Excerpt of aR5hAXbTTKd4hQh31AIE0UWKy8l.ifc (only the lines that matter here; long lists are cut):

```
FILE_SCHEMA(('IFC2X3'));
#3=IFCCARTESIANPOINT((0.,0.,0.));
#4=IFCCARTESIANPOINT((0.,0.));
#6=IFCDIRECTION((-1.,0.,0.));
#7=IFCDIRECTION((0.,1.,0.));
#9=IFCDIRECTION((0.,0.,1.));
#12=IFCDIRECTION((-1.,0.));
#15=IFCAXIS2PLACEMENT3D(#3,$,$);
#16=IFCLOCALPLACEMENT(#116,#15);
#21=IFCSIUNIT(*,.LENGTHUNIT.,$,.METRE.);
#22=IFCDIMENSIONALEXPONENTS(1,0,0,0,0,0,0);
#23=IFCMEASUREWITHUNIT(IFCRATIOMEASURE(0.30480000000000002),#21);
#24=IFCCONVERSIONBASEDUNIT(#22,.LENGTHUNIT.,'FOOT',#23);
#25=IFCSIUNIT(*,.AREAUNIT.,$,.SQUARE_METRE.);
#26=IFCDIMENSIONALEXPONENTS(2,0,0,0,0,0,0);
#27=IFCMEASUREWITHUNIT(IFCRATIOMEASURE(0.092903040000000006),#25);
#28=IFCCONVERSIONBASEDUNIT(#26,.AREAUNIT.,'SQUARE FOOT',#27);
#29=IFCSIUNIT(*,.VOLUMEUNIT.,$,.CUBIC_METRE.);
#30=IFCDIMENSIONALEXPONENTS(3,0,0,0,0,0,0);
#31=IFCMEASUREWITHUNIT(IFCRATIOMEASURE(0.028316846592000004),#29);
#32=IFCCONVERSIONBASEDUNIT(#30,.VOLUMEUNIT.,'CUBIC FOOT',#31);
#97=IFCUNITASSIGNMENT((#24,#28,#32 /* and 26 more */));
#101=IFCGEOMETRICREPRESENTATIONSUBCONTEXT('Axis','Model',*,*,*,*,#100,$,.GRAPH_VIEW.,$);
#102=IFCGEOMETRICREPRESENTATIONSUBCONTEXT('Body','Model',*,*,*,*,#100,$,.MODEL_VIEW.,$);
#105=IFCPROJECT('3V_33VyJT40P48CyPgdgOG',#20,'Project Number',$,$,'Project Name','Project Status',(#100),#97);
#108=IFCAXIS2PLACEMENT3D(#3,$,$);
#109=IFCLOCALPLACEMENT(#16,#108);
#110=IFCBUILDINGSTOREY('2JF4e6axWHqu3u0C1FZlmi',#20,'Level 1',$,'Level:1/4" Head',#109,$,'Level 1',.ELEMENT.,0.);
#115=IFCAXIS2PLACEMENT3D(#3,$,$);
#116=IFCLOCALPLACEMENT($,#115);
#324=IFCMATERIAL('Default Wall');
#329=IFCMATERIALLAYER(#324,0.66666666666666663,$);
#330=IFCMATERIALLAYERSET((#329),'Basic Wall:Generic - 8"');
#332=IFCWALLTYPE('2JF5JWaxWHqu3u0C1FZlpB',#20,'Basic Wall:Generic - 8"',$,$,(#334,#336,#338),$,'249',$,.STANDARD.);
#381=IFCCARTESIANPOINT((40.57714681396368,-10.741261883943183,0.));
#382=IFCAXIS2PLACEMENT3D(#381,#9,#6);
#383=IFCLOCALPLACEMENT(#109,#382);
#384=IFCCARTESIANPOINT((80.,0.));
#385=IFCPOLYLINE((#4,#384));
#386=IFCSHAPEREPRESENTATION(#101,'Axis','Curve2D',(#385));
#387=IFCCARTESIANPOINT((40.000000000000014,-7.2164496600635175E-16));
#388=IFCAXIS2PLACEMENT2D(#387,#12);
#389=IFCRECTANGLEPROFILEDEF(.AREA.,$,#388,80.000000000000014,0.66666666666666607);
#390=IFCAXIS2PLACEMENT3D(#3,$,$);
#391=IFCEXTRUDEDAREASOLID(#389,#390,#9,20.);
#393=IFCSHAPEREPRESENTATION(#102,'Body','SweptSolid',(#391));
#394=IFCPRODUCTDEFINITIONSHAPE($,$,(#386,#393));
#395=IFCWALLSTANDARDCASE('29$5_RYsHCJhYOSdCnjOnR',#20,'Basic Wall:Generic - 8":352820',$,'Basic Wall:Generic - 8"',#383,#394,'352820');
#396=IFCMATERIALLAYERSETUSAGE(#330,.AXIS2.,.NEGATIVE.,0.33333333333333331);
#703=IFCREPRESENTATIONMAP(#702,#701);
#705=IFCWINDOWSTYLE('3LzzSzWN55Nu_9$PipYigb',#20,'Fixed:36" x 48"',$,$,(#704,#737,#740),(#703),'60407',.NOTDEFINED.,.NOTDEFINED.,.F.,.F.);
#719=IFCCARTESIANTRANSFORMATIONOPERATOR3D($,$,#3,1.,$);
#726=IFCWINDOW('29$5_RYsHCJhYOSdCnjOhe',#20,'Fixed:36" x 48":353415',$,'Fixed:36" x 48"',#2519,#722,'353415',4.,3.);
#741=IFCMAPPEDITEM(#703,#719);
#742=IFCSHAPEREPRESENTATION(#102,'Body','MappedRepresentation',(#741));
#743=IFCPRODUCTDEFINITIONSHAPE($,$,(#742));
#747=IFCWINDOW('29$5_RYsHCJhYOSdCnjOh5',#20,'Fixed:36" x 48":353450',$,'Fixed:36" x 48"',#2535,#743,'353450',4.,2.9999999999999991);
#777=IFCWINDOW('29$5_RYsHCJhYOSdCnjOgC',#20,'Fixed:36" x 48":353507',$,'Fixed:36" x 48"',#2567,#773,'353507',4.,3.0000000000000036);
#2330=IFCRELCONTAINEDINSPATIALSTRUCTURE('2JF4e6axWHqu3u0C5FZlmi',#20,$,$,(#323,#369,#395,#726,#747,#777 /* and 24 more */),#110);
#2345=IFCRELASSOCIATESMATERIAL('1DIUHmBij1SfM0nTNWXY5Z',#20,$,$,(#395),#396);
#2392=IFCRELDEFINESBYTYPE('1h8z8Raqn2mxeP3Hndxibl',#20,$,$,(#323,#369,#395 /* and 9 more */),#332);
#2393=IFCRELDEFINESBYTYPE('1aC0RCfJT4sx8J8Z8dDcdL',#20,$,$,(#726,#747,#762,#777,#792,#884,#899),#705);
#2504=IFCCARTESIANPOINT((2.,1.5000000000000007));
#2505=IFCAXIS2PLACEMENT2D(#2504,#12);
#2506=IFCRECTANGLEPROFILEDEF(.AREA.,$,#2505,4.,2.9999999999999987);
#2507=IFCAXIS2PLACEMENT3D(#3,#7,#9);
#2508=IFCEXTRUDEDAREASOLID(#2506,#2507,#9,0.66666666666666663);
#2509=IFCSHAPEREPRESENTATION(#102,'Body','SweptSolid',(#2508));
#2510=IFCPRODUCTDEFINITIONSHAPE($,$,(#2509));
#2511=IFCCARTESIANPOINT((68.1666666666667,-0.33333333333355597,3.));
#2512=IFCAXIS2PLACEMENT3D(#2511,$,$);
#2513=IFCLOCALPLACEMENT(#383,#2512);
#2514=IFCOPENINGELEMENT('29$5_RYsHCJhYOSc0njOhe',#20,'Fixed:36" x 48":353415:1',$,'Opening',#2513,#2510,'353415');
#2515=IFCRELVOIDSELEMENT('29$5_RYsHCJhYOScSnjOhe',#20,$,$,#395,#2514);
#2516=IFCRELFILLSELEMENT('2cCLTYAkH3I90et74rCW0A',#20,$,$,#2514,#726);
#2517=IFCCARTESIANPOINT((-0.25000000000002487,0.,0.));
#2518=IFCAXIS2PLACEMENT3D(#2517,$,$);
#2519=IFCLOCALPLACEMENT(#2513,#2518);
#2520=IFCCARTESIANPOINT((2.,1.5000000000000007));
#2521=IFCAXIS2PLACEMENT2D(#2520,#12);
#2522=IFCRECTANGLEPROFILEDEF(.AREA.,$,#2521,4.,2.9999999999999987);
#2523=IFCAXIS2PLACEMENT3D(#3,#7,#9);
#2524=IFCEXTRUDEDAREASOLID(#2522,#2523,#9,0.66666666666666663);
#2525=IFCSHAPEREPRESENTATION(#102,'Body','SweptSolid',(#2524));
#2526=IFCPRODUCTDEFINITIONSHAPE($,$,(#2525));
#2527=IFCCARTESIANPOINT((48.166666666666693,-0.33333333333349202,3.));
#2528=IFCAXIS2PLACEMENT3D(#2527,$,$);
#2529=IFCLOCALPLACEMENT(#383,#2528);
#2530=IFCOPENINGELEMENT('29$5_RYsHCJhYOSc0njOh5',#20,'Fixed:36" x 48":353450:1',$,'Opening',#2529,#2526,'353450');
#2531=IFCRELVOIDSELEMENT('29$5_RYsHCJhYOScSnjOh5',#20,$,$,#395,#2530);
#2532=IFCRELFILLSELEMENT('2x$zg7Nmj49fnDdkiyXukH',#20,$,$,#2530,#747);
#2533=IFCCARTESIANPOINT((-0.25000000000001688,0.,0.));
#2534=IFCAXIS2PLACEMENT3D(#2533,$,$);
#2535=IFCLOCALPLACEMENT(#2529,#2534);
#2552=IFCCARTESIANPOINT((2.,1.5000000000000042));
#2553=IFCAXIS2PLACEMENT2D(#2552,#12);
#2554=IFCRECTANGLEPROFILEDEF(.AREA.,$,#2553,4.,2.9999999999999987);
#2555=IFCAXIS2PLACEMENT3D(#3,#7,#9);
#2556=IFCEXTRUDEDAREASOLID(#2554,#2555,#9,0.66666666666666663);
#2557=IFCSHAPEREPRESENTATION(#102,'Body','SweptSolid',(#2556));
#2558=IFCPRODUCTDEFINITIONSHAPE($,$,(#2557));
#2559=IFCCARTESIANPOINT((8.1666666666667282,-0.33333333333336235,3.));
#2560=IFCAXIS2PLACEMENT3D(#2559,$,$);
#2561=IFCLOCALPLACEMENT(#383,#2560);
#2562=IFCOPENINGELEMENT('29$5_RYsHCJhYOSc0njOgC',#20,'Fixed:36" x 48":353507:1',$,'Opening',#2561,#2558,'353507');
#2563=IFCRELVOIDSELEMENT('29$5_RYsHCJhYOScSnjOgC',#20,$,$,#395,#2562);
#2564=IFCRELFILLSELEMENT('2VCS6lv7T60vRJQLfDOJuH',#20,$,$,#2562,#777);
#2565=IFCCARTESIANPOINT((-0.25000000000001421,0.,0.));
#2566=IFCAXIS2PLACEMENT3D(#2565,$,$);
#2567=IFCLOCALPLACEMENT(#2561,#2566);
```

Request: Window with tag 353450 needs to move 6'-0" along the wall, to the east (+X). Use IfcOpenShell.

```python
import ifcopenshell
import ifcopenshell.api.geometry
import ifcopenshell.util.placement
import ifcopenshell.util.unit

model = ifcopenshell.open("aR5hAXbTTKd4hQh31AIE0UWKy8l.ifc")
unit_scale = ifcopenshell.util.unit.calculate_unit_scale(model)

window = model.by_id(747)
opening = window.FillsVoids[0].RelatingOpeningElement
wall = opening.VoidsElements[0].RelatingBuildingElement

wall_matrix = ifcopenshell.util.placement.get_local_placement(wall.ObjectPlacement)
shift = wall_matrix[:3, 0] * -72 * 0.0254 / unit_scale
before = ifcopenshell.util.placement.get_local_placement(window.ObjectPlacement)[:3, 3].copy()

# The window is placed relative to its opening, so it follows when the opening moves.
matrix = ifcopenshell.util.placement.get_local_placement(opening.ObjectPlacement)
matrix[:3, 3] += shift
ifcopenshell.api.geometry.edit_object_placement(
    model, product=opening, matrix=matrix, is_si=False, should_transform_children=True
)

after = ifcopenshell.util.placement.get_local_placement(window.ObjectPlacement)[:3, 3]
print("window moved by", (after - before).round(3) + 0.0)

model.write("aR5hAXbTTKd4hQh31AIE0UWKy8l-out.ifc")
```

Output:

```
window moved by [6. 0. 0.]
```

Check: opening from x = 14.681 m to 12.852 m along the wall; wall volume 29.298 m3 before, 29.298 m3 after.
